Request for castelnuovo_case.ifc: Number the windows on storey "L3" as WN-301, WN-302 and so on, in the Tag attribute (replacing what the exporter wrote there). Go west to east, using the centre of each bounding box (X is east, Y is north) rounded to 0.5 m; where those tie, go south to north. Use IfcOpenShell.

First a look at what the model holds.

```python
import ifcopenshell
import ifcopenshell.util.element
import ifcopenshell.util.placement

model = ifcopenshell.open("castelnuovo_case.ifc")
print(model.schema)
storey = next(s for s in model.by_type("IfcBuildingStorey") if s.Name == "L3")
windows = [e for e in ifcopenshell.util.element.get_decomposition(storey) if e.is_a("IfcWindow")]
for e in sorted(windows, key=lambda e: e.id()):
    origin = ifcopenshell.util.placement.get_local_placement(e.ObjectPlacement)[:3, 3]
    print(e.id(), e.Tag, e.Name, origin.round(2) + 0.0, sep=" | ")
```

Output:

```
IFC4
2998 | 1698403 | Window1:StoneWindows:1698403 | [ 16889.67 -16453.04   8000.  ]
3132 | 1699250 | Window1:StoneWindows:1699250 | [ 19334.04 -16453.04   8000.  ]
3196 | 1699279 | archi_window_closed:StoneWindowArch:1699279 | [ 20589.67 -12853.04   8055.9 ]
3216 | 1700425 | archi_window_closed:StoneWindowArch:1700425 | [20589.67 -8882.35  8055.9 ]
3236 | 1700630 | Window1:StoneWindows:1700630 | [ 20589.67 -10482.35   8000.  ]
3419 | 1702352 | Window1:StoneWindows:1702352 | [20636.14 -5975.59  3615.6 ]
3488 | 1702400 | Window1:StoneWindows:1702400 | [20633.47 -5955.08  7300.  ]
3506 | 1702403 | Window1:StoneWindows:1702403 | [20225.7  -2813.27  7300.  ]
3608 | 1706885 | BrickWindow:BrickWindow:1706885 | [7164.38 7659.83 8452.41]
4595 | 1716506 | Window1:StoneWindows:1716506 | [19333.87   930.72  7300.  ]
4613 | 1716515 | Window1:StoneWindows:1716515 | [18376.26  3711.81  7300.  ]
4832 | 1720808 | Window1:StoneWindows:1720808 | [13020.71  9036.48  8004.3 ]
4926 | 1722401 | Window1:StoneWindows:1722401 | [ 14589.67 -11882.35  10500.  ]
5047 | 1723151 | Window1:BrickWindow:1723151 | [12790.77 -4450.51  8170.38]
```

```python
import ifcopenshell
import ifcopenshell.geom
import ifcopenshell.util.element
import ifcopenshell.util.shape

model = ifcopenshell.open("castelnuovo_case.ifc")
settings = ifcopenshell.geom.settings()
settings.set("use-world-coords", True)


def centre(element):
    shape = ifcopenshell.geom.create_shape(settings, element)
    return ifcopenshell.util.shape.get_bbox_centroid(shape.geometry)


storey = next(s for s in model.by_type("IfcBuildingStorey") if s.Name == "L3")
windows = [e for e in ifcopenshell.util.element.get_decomposition(storey) if e.is_a("IfcWindow")]

# Insertion points can sit at a corner or the storey origin, so sort by the geometry (in metres).
centres = {e: centre(e) for e in windows}
windows.sort(key=lambda e: (round(centres[e][0] / 0.5), centres[e][1]))

for i, e in enumerate(windows, start=1):
    number = f"WN-3{i:02d}"
    e.Tag = number
    print(e.id(), number)

model.write("castelnuovo_case-out.ifc")
```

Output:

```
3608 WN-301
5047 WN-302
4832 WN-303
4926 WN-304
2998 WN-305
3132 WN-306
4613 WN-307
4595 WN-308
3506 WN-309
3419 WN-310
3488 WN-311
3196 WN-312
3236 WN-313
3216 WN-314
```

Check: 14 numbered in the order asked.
